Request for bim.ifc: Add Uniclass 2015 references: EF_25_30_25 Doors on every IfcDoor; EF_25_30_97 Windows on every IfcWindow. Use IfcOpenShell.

First a look at what the model holds.

```python
import ifcopenshell

model = ifcopenshell.open("bim.ifc")
print(model.schema)
print("classifications:", [c.Name for c in model.by_type("IfcClassification")])
for ifc_class in ("IfcDoor", "IfcRoof", "IfcStair", "IfcWall", "IfcWindow"):
    print(ifc_class, len(model.by_type(ifc_class)))
```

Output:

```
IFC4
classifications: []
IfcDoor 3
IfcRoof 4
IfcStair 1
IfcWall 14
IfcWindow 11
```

```python
import ifcopenshell
import ifcopenshell.api.classification

model = ifcopenshell.open("bim.ifc")

system = ifcopenshell.api.classification.add_classification(model, classification="Uniclass 2015")

codes = {
    "IfcDoor": ("EF_25_30_25", "Doors"),
    "IfcWindow": ("EF_25_30_97", "Windows"),
}
for ifc_class, (code, name) in codes.items():
    products = model.by_type(ifc_class)
    ifcopenshell.api.classification.add_reference(
        model, products=products, classification=system, identification=code, name=name
    )
    print(code, len(products))

model.write("bim_updated.ifc")
```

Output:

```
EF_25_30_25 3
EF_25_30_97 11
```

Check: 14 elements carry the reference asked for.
